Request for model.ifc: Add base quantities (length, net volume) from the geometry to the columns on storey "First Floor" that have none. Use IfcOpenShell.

First a look at what the model holds.

```python
import ifcopenshell
import ifcopenshell.util.element
import ifcopenshell.util.unit

model = ifcopenshell.open("model.ifc")
print(model.schema)
for unit_type in ("LENGTHUNIT", "AREAUNIT", "VOLUMEUNIT"):
    print(unit_type, ifcopenshell.util.unit.calculate_unit_scale(model, unit_type))
storey = next(s for s in model.by_type("IfcBuildingStorey") if s.Name == "First Floor")
columns = [e for e in ifcopenshell.util.element.get_decomposition(storey) if e.is_a("IfcColumn")]
for e in sorted(columns, key=lambda e: e.id()):
    print(e.id(), e.is_a(), e.Name, list(ifcopenshell.util.element.get_psets(e, qtos_only=True)), sep=" | ")
```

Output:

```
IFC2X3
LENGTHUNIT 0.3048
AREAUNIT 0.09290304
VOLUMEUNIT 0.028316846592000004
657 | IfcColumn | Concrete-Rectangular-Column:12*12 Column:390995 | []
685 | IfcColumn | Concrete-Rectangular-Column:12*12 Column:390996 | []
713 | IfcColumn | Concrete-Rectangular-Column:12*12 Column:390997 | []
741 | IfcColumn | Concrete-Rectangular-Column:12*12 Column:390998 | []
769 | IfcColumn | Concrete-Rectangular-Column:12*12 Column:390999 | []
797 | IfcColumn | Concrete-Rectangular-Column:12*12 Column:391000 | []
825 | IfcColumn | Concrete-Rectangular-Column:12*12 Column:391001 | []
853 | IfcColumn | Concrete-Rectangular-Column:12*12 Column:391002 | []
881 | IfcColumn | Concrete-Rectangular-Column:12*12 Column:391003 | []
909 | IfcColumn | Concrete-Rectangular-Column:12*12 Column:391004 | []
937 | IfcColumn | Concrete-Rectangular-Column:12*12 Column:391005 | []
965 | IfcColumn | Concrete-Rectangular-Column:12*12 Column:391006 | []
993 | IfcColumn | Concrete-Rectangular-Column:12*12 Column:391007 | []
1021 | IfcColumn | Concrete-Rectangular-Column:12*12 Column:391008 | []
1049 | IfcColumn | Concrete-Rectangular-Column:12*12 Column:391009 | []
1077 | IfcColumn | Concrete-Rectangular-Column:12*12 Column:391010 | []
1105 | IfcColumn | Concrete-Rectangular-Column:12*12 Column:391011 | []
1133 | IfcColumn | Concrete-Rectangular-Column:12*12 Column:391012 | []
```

```python
import ifcopenshell
import ifcopenshell.api.pset
import ifcopenshell.geom
import ifcopenshell.util.element
import ifcopenshell.util.shape
import ifcopenshell.util.unit

model = ifcopenshell.open("model.ifc")
unit_scale = ifcopenshell.util.unit.calculate_unit_scale(model)
volume_scale = ifcopenshell.util.unit.calculate_unit_scale(model, "VOLUMEUNIT")
settings = ifcopenshell.geom.settings()

storey = next(s for s in model.by_type("IfcBuildingStorey") if s.Name == "First Floor")
columns = [e for e in ifcopenshell.util.element.get_decomposition(storey) if e.is_a("IfcColumn")]

for e in sorted(columns, key=lambda e: e.id()):
    if ifcopenshell.util.element.get_psets(e, qtos_only=True, should_inherit=False):
        continue
    # Geometry comes back in metres, in the element's own axes.
    shape = ifcopenshell.geom.create_shape(settings, e)
    values = {
        "Length": ifcopenshell.util.shape.get_z(shape.geometry) / unit_scale,
        "NetVolume": ifcopenshell.util.shape.get_volume(shape.geometry) / volume_scale,
    }
    qto = ifcopenshell.api.pset.add_qto(model, product=e, name="BaseQuantities")
    ifcopenshell.api.pset.edit_qto(model, qto=qto, properties=values)
    print(e.id(), {k: round(v, 3) for k, v in values.items()})

model.write("model_updated.ifc")
```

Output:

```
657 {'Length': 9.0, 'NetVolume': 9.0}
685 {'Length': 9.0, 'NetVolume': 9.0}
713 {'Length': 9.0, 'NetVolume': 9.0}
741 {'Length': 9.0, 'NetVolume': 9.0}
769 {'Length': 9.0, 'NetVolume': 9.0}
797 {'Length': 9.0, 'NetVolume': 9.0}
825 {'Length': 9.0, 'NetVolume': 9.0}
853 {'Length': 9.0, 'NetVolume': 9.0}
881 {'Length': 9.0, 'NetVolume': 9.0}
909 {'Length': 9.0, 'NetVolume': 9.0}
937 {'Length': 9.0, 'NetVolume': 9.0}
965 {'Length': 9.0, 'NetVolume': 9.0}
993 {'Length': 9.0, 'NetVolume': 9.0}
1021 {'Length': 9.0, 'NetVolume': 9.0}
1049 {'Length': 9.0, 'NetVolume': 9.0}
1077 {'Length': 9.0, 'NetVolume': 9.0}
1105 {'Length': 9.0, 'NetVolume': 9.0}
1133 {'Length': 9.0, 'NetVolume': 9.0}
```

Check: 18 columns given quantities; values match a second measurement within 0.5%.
